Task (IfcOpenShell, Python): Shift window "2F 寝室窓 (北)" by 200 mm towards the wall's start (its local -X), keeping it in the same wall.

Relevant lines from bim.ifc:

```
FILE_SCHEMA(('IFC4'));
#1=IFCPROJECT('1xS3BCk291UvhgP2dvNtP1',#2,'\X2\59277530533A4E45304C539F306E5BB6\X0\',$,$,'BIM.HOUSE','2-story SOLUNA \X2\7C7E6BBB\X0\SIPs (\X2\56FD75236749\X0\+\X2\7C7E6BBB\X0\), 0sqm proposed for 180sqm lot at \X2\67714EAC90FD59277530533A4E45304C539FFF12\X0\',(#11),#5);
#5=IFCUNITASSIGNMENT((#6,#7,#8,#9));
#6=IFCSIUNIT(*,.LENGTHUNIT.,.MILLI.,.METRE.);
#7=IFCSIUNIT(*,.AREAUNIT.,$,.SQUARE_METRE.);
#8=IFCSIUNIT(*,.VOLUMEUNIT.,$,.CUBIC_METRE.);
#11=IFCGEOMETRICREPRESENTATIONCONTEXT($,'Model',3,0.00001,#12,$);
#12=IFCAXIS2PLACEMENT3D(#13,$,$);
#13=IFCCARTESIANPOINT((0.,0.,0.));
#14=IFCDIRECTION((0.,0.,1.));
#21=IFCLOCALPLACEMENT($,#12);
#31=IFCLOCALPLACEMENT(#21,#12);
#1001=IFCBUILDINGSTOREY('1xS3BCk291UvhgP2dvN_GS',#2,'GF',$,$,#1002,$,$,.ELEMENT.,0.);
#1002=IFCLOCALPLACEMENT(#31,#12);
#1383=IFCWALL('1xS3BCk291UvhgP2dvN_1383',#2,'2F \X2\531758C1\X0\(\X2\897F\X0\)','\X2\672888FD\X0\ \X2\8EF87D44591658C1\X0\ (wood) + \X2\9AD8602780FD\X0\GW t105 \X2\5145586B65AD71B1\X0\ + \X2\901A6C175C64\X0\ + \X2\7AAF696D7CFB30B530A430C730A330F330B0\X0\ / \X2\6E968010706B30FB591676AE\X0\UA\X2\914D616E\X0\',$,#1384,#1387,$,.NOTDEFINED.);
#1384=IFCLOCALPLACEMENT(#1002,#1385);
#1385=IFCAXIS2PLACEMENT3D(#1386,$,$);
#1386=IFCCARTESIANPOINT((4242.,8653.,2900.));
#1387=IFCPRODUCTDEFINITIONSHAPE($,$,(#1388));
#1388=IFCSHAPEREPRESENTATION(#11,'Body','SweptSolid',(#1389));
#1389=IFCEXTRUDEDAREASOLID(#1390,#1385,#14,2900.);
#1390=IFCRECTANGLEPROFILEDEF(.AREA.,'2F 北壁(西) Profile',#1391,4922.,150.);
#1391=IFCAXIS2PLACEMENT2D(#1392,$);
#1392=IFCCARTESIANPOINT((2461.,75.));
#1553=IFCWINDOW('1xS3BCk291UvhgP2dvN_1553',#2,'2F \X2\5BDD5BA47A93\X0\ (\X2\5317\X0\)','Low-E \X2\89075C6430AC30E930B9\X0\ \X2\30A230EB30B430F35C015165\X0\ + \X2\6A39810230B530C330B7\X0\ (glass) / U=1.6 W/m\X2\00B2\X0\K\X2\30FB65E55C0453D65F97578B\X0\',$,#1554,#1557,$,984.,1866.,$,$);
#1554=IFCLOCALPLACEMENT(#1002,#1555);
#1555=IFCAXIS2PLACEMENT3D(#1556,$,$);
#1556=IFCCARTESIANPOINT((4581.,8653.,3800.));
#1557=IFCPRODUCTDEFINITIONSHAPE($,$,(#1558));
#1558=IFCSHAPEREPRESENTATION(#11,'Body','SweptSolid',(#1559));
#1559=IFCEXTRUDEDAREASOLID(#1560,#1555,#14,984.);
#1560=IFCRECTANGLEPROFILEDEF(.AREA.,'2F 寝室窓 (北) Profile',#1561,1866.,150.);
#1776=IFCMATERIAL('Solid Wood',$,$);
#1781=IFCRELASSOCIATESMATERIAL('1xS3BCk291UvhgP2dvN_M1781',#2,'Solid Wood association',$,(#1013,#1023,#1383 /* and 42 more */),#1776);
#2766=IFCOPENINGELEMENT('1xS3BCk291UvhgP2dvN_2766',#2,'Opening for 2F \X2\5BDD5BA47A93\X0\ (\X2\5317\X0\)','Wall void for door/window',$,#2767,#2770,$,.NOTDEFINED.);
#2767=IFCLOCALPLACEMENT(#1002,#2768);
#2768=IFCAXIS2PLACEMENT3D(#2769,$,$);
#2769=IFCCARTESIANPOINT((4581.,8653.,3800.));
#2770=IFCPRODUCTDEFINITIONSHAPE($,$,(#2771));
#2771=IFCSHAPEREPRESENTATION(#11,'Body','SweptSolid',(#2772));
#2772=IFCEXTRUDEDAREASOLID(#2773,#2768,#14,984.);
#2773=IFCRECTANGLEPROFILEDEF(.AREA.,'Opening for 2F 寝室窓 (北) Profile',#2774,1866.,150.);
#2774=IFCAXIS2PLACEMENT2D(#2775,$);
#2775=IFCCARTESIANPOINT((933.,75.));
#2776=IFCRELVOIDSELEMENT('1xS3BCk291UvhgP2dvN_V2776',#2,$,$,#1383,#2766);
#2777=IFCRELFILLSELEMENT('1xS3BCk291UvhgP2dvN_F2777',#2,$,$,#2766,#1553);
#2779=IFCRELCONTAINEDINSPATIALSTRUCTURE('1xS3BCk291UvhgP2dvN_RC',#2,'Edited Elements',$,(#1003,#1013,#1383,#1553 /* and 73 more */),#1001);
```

```python
import ifcopenshell
import ifcopenshell.api.geometry
import ifcopenshell.util.placement
import ifcopenshell.util.unit

model = ifcopenshell.open("bim.ifc")
unit_scale = ifcopenshell.util.unit.calculate_unit_scale(model)

window = model.by_guid("1xS3BCk291UvhgP2dvN_1553")
opening = window.FillsVoids[0].RelatingOpeningElement
wall = opening.VoidsElements[0].RelatingBuildingElement

wall_matrix = ifcopenshell.util.placement.get_local_placement(wall.ObjectPlacement)
shift = wall_matrix[:3, 0] * -0.2 / unit_scale
before = ifcopenshell.util.placement.get_local_placement(window.ObjectPlacement)[:3, 3].copy()

# The window is not placed relative to its opening, so move both.
for product in (opening, window):
    matrix = ifcopenshell.util.placement.get_local_placement(product.ObjectPlacement)
    matrix[:3, 3] += shift
    ifcopenshell.api.geometry.edit_object_placement(model, product=product, matrix=matrix, is_si=False)

after = ifcopenshell.util.placement.get_local_placement(window.ObjectPlacement)[:3, 3]
print("window moved by", (after - before).round(3) + 0.0)

model.write("bim_updated.ifc")
```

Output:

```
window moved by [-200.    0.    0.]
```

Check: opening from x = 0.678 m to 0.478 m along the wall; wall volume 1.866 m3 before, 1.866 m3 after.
